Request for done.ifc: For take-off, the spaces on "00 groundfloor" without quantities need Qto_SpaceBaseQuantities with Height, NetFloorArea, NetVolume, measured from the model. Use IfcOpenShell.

First a look at what the model holds.

```python
import ifcopenshell
import ifcopenshell.util.element
import ifcopenshell.util.unit

model = ifcopenshell.open("done.ifc")
print(model.schema)
for unit_type in ("LENGTHUNIT", "AREAUNIT", "VOLUMEUNIT"):
    print(unit_type, ifcopenshell.util.unit.calculate_unit_scale(model, unit_type))
storey = next(s for s in model.by_type("IfcBuildingStorey") if s.Name == "00 groundfloor")
spaces = [e for e in ifcopenshell.util.element.get_decomposition(storey) if e.is_a("IfcSpace")]
for e in sorted(spaces, key=lambda e: e.id()):
    print(e.id(), e.is_a(), e.Name, list(ifcopenshell.util.element.get_psets(e, qtos_only=True)), sep=" | ")
```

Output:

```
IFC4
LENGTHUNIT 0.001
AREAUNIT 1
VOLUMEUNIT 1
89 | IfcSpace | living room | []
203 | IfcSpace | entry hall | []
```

```python
import ifcopenshell
import ifcopenshell.api.pset
import ifcopenshell.geom
import ifcopenshell.util.element
import ifcopenshell.util.shape
import ifcopenshell.util.unit

model = ifcopenshell.open("done.ifc")
unit_scale = ifcopenshell.util.unit.calculate_unit_scale(model)
area_scale = ifcopenshell.util.unit.calculate_unit_scale(model, "AREAUNIT")
volume_scale = ifcopenshell.util.unit.calculate_unit_scale(model, "VOLUMEUNIT")
settings = ifcopenshell.geom.settings()

storey = next(s for s in model.by_type("IfcBuildingStorey") if s.Name == "00 groundfloor")
spaces = [e for e in ifcopenshell.util.element.get_decomposition(storey) if e.is_a("IfcSpace")]

for e in sorted(spaces, key=lambda e: e.id()):
    if ifcopenshell.util.element.get_psets(e, qtos_only=True, should_inherit=False):
        continue
    # Geometry comes back in metres, in the element's own axes.
    shape = ifcopenshell.geom.create_shape(settings, e)
    values = {
        "Height": ifcopenshell.util.shape.get_z(shape.geometry) / unit_scale,
        "NetFloorArea": ifcopenshell.util.shape.get_footprint_area(shape.geometry) / area_scale,
        "NetVolume": ifcopenshell.util.shape.get_volume(shape.geometry) / volume_scale,
    }
    qto = ifcopenshell.api.pset.add_qto(model, product=e, name="Qto_SpaceBaseQuantities")
    ifcopenshell.api.pset.edit_qto(model, qto=qto, properties=values)
    print(e.id(), {k: round(v, 3) for k, v in values.items()})

model.write("done_rev.ifc")
```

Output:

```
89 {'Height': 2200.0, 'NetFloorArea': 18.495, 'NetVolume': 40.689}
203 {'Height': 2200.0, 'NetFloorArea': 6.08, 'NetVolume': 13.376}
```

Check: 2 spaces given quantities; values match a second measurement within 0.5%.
